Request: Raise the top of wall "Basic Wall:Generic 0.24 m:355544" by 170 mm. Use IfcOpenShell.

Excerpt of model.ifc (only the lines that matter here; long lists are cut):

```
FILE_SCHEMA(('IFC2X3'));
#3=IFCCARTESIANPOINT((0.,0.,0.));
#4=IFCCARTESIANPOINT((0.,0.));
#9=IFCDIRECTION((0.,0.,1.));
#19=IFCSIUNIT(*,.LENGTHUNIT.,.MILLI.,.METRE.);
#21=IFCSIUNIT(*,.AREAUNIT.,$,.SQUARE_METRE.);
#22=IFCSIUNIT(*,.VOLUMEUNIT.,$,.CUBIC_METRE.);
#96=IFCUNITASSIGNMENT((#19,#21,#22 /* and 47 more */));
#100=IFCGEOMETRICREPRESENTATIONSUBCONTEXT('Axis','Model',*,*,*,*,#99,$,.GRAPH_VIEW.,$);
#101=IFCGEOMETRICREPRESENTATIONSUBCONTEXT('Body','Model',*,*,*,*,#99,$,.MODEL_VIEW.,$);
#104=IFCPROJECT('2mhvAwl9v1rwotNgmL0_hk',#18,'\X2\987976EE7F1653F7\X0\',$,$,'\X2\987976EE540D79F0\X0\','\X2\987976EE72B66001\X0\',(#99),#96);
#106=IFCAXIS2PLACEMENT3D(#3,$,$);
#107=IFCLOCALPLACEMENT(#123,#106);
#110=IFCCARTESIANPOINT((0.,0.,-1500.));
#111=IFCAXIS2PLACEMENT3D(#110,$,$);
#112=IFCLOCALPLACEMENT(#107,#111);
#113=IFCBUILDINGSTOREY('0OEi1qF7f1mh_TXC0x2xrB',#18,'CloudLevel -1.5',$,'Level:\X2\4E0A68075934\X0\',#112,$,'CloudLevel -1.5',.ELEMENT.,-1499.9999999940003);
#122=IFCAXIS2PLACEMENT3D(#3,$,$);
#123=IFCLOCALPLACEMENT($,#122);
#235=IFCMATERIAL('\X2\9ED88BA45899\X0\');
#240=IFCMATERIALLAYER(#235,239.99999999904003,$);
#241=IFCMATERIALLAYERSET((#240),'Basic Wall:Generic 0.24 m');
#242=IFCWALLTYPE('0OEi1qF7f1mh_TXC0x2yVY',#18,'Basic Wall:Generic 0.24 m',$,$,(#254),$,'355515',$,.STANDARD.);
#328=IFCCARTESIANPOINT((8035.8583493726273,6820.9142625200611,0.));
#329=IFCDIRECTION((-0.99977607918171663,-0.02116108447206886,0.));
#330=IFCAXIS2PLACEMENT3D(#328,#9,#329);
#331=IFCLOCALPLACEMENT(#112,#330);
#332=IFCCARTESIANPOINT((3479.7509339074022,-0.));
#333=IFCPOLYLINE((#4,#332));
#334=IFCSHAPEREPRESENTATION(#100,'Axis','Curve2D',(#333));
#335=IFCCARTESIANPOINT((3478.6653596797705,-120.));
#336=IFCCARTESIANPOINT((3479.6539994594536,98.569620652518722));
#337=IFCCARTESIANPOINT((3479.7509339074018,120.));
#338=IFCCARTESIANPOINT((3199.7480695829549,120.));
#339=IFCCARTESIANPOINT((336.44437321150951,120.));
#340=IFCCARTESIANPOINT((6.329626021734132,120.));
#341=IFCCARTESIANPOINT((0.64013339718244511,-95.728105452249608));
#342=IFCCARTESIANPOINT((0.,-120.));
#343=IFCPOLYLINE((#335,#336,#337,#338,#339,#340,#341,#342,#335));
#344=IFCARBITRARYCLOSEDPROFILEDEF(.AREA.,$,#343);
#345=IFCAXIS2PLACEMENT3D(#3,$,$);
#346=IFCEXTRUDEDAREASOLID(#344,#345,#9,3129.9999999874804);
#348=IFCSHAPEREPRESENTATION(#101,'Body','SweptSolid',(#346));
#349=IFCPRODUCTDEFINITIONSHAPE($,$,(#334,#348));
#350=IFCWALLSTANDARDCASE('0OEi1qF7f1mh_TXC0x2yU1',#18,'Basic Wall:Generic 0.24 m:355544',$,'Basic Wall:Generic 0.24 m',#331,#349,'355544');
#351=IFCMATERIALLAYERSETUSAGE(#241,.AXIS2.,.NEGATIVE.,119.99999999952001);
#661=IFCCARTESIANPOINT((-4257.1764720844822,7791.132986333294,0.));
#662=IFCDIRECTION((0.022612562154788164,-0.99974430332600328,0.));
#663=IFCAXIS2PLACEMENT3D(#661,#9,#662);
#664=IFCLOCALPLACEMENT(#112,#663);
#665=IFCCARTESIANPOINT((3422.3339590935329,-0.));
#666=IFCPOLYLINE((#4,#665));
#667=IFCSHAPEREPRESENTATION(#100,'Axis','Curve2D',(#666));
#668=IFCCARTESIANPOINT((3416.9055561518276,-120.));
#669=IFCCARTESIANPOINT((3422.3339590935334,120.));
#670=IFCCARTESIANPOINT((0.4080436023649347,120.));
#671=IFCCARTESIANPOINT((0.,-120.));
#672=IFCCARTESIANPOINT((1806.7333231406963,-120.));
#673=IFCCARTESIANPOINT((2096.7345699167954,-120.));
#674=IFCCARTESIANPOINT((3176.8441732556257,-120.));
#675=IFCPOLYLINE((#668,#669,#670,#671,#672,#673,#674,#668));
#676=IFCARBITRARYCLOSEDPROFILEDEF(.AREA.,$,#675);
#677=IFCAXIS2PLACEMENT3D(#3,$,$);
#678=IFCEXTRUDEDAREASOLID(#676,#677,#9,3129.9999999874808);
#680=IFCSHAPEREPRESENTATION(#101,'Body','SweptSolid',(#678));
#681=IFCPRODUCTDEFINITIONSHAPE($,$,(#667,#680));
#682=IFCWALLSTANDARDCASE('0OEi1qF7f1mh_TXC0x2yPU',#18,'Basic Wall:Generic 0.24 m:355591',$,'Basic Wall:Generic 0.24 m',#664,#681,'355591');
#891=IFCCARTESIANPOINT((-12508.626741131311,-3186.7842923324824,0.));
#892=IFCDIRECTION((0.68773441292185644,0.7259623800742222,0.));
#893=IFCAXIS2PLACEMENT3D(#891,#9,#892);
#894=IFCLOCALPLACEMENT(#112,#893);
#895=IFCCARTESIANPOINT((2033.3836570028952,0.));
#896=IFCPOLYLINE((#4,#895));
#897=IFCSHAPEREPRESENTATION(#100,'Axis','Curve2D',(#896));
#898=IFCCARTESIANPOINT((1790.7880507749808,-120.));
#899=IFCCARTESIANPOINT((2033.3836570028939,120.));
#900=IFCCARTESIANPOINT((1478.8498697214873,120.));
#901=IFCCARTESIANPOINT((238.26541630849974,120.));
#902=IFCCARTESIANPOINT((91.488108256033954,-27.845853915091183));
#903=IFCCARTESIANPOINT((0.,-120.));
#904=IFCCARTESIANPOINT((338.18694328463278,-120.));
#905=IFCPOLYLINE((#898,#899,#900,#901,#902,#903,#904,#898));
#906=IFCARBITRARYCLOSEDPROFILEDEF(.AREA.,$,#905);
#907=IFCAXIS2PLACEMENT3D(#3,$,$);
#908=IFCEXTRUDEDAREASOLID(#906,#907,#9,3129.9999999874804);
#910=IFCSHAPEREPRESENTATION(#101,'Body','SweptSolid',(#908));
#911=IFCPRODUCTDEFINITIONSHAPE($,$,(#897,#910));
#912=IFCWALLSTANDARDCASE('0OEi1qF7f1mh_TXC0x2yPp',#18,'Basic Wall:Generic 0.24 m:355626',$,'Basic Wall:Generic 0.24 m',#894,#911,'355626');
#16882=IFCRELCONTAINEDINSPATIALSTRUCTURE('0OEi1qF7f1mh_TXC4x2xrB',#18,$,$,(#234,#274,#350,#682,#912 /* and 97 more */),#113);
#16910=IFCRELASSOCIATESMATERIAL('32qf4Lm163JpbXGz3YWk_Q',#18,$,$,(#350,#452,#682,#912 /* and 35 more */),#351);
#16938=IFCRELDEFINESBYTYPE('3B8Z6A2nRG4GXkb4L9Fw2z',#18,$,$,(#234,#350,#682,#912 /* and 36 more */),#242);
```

```python
import ifcopenshell
import ifcopenshell.geom
import ifcopenshell.util.representation
import ifcopenshell.util.shape

model = ifcopenshell.open("model.ifc")
settings = ifcopenshell.geom.settings()


def volume(element):
    """Net volume in cubic metres, openings subtracted."""
    shape = ifcopenshell.geom.create_shape(settings, element)
    return ifcopenshell.util.shape.get_volume(shape.geometry)


wall = model.by_id(350)
before = volume(wall)

body = ifcopenshell.util.representation.get_representation(wall, "Model", "Body")
solid = body.Items[0]
old_height = solid.Depth
solid.Depth += 170.0
after = volume(wall)

print(f"height {old_height:g} -> {solid.Depth:g}, volume {before:.3f} -> {after:.3f} m3")

model.write("model_v2.ifc")
```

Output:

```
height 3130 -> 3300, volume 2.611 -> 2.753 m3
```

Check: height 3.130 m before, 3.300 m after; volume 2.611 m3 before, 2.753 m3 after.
